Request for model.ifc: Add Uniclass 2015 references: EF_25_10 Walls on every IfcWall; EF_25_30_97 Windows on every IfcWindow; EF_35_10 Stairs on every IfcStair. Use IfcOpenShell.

First a look at what the model holds.

```python
import ifcopenshell

model = ifcopenshell.open("model.ifc")
print(model.schema)
print("classifications:", [c.Name for c in model.by_type("IfcClassification")])
for ifc_class in ("IfcDoor", "IfcRoof", "IfcStair", "IfcWall", "IfcWindow"):
    print(ifc_class, len(model.by_type(ifc_class)))
```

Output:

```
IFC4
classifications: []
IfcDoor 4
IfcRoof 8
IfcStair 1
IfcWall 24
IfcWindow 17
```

```python
import ifcopenshell
import ifcopenshell.api.classification

model = ifcopenshell.open("model.ifc")

system = ifcopenshell.api.classification.add_classification(model, classification="Uniclass 2015")

codes = {
    "IfcWall": ("EF_25_10", "Walls"),
    "IfcWindow": ("EF_25_30_97", "Windows"),
    "IfcStair": ("EF_35_10", "Stairs"),
}
for ifc_class, (code, name) in codes.items():
    products = model.by_type(ifc_class)
    ifcopenshell.api.classification.add_reference(
        model, products=products, classification=system, identification=code, name=name
    )
    print(code, len(products))

model.write("model_edited.ifc")
```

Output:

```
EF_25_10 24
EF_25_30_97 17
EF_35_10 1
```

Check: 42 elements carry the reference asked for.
